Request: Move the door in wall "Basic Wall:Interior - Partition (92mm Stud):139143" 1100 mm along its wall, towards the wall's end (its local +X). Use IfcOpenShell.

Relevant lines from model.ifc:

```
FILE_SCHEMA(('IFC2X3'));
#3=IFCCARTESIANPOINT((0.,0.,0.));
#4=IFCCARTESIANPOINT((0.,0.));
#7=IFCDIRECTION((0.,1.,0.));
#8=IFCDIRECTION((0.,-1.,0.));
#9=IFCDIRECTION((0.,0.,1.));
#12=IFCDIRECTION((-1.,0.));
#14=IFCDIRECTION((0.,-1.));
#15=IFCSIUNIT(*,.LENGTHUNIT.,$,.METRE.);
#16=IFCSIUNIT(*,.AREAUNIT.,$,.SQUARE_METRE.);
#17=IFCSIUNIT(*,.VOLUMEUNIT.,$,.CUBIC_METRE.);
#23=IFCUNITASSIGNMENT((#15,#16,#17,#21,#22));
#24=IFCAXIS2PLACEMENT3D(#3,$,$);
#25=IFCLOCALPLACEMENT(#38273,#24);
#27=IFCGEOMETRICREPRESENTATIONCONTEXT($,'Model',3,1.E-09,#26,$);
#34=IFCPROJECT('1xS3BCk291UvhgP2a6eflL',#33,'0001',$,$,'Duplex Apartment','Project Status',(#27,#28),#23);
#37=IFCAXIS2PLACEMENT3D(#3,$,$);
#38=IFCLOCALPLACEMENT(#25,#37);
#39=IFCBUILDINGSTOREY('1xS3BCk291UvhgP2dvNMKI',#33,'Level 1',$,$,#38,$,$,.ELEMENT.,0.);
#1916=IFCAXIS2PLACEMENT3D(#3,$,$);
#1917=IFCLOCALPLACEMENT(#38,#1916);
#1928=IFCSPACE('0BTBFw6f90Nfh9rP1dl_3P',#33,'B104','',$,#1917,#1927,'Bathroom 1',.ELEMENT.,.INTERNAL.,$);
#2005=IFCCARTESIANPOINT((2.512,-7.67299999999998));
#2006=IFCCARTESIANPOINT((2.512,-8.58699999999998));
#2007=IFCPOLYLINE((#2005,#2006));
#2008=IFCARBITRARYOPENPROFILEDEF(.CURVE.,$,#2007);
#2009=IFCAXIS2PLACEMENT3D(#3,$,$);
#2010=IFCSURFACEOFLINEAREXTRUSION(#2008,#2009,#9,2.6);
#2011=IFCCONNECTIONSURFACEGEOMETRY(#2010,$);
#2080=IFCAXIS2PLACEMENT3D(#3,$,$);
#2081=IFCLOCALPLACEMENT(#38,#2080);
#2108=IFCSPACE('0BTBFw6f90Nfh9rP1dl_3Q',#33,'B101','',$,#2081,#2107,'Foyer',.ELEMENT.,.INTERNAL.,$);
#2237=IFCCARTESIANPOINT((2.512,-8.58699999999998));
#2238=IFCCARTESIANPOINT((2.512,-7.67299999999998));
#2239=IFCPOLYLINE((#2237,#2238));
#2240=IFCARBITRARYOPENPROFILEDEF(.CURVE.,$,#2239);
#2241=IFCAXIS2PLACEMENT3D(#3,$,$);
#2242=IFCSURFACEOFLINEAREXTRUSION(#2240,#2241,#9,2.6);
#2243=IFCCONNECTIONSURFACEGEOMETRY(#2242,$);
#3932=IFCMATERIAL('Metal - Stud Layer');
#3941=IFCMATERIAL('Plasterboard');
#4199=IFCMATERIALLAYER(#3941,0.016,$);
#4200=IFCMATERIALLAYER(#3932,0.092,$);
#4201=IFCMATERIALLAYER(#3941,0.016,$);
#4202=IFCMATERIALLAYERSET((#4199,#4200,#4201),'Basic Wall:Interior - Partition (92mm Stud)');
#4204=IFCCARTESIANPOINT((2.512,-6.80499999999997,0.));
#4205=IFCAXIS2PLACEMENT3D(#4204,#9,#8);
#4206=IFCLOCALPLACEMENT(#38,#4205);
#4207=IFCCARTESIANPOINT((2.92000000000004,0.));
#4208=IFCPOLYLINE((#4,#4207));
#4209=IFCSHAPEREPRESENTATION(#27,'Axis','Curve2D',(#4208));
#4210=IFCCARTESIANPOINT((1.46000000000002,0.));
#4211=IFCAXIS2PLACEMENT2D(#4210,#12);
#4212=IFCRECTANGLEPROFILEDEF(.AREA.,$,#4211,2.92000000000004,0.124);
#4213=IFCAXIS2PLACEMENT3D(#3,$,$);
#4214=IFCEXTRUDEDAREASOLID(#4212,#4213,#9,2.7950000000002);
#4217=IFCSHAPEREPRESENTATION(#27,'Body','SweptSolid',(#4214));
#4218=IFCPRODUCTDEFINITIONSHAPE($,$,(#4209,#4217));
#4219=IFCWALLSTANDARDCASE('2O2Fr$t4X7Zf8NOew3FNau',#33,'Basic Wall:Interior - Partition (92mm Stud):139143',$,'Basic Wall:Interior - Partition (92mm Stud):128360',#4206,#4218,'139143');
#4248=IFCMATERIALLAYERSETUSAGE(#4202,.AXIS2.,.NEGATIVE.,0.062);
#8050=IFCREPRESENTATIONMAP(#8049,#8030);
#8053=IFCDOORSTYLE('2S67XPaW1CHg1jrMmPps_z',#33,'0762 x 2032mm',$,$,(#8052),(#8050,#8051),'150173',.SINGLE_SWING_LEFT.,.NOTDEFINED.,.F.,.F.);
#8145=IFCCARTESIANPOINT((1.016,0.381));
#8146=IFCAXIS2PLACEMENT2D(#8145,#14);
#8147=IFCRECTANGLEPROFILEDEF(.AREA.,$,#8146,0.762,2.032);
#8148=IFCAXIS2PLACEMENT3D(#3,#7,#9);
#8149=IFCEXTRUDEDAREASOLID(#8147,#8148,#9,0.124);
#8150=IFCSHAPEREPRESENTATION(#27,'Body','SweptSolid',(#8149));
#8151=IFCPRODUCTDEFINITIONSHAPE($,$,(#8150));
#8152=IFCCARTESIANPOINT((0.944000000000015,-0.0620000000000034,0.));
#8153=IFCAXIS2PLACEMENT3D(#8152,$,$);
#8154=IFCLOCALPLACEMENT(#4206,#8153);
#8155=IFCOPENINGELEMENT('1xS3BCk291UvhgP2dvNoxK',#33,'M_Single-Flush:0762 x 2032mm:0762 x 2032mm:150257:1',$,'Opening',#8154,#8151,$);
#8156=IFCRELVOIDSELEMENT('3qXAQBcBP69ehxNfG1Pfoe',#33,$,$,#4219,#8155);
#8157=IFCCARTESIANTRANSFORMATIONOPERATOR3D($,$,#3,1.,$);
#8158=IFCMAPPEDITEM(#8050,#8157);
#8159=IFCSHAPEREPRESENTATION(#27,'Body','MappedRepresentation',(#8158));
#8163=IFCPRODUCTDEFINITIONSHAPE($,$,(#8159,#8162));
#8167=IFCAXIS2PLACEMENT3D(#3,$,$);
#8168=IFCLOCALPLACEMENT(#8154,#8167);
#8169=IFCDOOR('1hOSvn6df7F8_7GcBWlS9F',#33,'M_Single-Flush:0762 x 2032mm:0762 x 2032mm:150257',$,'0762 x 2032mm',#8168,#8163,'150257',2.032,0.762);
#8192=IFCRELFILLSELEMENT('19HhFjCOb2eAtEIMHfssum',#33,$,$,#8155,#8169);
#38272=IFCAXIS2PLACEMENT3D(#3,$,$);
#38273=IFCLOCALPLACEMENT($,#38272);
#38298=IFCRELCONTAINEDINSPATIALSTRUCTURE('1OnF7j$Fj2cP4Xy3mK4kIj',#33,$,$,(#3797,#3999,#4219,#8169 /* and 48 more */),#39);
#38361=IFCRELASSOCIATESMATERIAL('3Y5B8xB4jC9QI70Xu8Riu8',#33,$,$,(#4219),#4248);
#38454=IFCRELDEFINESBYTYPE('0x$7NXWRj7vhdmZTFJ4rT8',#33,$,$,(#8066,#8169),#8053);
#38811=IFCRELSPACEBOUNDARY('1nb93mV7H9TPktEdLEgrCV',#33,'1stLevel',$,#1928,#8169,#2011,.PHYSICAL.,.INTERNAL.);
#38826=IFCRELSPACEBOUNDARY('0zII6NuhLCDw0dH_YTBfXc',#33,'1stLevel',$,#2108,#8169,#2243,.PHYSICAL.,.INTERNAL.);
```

```python
import numpy as np
import ifcopenshell
import ifcopenshell.api.geometry
import ifcopenshell.util.placement
import ifcopenshell.util.unit

model = ifcopenshell.open("model.ifc")
unit_scale = ifcopenshell.util.unit.calculate_unit_scale(model)

door = model.by_guid("1hOSvn6df7F8_7GcBWlS9F")
opening = door.FillsVoids[0].RelatingOpeningElement
wall = opening.VoidsElements[0].RelatingBuildingElement

wall_matrix = ifcopenshell.util.placement.get_local_placement(wall.ObjectPlacement)
shift = wall_matrix[:3, 0] * 1.1 / unit_scale
before = ifcopenshell.util.placement.get_local_placement(door.ObjectPlacement)[:3, 3].copy()

# The door is placed relative to its opening, so it follows when the opening moves.
matrix = ifcopenshell.util.placement.get_local_placement(opening.ObjectPlacement)
matrix[:3, 3] += shift
ifcopenshell.api.geometry.edit_object_placement(
    model, product=opening, matrix=matrix, is_si=False, should_transform_children=True
)

# Space boundary surfaces are stored in each space's coordinates; move them too.
for rel in door.ProvidesBoundaries:
    if not rel.ConnectionGeometry:
        continue
    surface = rel.ConnectionGeometry.SurfaceOnRelatingElement
    space_matrix = ifcopenshell.util.placement.get_local_placement(rel.RelatingSpace.ObjectPlacement)
    point = np.array(surface.Position.Location.Coordinates) + space_matrix[:3, :3].T @ shift
    surface.Position = model.createIfcAxis2Placement3D(
        model.createIfcCartesianPoint(point.tolist()), surface.Position.Axis, surface.Position.RefDirection
    )

after = ifcopenshell.util.placement.get_local_placement(door.ObjectPlacement)[:3, 3]
print("door moved by", (after - before).round(3) + 0.0)

model.write("model_rev.ifc")
```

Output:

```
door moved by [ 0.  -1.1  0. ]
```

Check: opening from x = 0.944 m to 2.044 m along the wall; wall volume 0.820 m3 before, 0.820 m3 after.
